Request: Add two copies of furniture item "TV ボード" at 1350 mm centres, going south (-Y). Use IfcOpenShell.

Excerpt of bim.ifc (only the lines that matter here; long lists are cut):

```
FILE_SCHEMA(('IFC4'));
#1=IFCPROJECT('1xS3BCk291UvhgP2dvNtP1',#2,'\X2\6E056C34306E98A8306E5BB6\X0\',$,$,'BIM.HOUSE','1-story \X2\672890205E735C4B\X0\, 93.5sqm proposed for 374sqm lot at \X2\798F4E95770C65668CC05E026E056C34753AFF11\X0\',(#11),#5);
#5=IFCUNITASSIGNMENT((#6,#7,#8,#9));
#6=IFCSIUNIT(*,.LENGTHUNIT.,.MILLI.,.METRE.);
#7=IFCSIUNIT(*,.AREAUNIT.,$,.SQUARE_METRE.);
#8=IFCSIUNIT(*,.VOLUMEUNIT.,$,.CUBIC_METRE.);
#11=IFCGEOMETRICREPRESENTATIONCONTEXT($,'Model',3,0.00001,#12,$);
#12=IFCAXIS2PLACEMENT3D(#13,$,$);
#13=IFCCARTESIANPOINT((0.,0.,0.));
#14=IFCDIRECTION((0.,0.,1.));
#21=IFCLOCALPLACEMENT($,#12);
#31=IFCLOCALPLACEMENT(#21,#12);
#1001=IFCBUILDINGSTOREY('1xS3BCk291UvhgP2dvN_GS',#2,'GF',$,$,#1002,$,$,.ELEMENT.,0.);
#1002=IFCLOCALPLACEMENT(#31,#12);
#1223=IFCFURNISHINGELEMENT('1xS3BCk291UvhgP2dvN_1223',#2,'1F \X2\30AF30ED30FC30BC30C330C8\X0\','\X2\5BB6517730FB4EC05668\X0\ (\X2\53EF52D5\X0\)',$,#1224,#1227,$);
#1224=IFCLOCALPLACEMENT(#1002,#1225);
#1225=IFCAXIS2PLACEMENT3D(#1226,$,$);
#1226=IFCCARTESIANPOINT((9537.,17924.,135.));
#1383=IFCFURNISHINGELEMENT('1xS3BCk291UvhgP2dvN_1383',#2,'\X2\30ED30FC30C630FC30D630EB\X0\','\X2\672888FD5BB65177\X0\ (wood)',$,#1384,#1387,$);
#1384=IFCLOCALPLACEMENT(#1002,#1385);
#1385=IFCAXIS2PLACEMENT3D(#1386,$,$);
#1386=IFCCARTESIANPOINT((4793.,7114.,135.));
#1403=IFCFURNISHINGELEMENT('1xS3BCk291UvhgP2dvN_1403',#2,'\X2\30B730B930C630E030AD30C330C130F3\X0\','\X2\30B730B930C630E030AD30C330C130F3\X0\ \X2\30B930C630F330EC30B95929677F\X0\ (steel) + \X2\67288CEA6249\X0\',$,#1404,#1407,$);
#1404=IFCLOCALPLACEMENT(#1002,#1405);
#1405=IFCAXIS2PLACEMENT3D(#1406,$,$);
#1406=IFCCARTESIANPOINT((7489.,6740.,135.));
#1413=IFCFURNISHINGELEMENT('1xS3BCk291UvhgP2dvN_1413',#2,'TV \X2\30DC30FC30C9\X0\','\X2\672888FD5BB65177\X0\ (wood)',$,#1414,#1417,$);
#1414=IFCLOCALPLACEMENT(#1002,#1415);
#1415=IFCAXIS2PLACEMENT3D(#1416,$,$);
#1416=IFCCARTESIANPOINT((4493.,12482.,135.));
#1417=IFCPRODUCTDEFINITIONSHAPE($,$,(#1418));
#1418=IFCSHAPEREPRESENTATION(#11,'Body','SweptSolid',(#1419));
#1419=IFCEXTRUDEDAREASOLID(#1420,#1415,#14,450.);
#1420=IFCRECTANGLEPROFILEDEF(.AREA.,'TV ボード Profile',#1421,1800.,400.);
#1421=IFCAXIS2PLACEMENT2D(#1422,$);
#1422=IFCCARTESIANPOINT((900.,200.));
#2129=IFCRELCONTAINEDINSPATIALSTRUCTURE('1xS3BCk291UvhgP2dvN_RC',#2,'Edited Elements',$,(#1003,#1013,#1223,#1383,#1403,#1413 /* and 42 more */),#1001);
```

```python
import numpy as np
import ifcopenshell
import ifcopenshell.api.geometry
import ifcopenshell.api.root
import ifcopenshell.util.element
import ifcopenshell.util.placement

model = ifcopenshell.open("bim.ifc")


def reuse_history(source, copy):
    """copy_class also copies each property set's owner history, people and application; keep the originals."""
    for rel in copy.IsDefinedBy:
        if rel.is_a("IfcRelDefinesByProperties") and (history := rel.RelatingPropertyDefinition.OwnerHistory):
            rel.RelatingPropertyDefinition.OwnerHistory = source.OwnerHistory
            ifcopenshell.util.element.remove_deep2(model, history)


source = model.by_guid("1xS3BCk291UvhgP2dvN_1413")
base = ifcopenshell.util.placement.get_local_placement(source.ObjectPlacement)
step = np.array([0.0, -1.0, 0.0]) * 1350.0

for i in range(1, 3):
    copy = ifcopenshell.api.root.copy_class(model, product=source)
    copy.Representation = ifcopenshell.util.element.copy_deep(
        model, source.Representation, exclude=["IfcGeometricRepresentationContext", "IfcRepresentationMap"]
    )
    reuse_history(source, copy)
    matrix = base.copy()
    matrix[:3, 3] += i * step
    print("added at", matrix[:3, 3].round(3) + 0.0)
    ifcopenshell.api.geometry.edit_object_placement(model, product=copy, matrix=matrix, is_si=False)

model.write("bim_updated.ifc")
```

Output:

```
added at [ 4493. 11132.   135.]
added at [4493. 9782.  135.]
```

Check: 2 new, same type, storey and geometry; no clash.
